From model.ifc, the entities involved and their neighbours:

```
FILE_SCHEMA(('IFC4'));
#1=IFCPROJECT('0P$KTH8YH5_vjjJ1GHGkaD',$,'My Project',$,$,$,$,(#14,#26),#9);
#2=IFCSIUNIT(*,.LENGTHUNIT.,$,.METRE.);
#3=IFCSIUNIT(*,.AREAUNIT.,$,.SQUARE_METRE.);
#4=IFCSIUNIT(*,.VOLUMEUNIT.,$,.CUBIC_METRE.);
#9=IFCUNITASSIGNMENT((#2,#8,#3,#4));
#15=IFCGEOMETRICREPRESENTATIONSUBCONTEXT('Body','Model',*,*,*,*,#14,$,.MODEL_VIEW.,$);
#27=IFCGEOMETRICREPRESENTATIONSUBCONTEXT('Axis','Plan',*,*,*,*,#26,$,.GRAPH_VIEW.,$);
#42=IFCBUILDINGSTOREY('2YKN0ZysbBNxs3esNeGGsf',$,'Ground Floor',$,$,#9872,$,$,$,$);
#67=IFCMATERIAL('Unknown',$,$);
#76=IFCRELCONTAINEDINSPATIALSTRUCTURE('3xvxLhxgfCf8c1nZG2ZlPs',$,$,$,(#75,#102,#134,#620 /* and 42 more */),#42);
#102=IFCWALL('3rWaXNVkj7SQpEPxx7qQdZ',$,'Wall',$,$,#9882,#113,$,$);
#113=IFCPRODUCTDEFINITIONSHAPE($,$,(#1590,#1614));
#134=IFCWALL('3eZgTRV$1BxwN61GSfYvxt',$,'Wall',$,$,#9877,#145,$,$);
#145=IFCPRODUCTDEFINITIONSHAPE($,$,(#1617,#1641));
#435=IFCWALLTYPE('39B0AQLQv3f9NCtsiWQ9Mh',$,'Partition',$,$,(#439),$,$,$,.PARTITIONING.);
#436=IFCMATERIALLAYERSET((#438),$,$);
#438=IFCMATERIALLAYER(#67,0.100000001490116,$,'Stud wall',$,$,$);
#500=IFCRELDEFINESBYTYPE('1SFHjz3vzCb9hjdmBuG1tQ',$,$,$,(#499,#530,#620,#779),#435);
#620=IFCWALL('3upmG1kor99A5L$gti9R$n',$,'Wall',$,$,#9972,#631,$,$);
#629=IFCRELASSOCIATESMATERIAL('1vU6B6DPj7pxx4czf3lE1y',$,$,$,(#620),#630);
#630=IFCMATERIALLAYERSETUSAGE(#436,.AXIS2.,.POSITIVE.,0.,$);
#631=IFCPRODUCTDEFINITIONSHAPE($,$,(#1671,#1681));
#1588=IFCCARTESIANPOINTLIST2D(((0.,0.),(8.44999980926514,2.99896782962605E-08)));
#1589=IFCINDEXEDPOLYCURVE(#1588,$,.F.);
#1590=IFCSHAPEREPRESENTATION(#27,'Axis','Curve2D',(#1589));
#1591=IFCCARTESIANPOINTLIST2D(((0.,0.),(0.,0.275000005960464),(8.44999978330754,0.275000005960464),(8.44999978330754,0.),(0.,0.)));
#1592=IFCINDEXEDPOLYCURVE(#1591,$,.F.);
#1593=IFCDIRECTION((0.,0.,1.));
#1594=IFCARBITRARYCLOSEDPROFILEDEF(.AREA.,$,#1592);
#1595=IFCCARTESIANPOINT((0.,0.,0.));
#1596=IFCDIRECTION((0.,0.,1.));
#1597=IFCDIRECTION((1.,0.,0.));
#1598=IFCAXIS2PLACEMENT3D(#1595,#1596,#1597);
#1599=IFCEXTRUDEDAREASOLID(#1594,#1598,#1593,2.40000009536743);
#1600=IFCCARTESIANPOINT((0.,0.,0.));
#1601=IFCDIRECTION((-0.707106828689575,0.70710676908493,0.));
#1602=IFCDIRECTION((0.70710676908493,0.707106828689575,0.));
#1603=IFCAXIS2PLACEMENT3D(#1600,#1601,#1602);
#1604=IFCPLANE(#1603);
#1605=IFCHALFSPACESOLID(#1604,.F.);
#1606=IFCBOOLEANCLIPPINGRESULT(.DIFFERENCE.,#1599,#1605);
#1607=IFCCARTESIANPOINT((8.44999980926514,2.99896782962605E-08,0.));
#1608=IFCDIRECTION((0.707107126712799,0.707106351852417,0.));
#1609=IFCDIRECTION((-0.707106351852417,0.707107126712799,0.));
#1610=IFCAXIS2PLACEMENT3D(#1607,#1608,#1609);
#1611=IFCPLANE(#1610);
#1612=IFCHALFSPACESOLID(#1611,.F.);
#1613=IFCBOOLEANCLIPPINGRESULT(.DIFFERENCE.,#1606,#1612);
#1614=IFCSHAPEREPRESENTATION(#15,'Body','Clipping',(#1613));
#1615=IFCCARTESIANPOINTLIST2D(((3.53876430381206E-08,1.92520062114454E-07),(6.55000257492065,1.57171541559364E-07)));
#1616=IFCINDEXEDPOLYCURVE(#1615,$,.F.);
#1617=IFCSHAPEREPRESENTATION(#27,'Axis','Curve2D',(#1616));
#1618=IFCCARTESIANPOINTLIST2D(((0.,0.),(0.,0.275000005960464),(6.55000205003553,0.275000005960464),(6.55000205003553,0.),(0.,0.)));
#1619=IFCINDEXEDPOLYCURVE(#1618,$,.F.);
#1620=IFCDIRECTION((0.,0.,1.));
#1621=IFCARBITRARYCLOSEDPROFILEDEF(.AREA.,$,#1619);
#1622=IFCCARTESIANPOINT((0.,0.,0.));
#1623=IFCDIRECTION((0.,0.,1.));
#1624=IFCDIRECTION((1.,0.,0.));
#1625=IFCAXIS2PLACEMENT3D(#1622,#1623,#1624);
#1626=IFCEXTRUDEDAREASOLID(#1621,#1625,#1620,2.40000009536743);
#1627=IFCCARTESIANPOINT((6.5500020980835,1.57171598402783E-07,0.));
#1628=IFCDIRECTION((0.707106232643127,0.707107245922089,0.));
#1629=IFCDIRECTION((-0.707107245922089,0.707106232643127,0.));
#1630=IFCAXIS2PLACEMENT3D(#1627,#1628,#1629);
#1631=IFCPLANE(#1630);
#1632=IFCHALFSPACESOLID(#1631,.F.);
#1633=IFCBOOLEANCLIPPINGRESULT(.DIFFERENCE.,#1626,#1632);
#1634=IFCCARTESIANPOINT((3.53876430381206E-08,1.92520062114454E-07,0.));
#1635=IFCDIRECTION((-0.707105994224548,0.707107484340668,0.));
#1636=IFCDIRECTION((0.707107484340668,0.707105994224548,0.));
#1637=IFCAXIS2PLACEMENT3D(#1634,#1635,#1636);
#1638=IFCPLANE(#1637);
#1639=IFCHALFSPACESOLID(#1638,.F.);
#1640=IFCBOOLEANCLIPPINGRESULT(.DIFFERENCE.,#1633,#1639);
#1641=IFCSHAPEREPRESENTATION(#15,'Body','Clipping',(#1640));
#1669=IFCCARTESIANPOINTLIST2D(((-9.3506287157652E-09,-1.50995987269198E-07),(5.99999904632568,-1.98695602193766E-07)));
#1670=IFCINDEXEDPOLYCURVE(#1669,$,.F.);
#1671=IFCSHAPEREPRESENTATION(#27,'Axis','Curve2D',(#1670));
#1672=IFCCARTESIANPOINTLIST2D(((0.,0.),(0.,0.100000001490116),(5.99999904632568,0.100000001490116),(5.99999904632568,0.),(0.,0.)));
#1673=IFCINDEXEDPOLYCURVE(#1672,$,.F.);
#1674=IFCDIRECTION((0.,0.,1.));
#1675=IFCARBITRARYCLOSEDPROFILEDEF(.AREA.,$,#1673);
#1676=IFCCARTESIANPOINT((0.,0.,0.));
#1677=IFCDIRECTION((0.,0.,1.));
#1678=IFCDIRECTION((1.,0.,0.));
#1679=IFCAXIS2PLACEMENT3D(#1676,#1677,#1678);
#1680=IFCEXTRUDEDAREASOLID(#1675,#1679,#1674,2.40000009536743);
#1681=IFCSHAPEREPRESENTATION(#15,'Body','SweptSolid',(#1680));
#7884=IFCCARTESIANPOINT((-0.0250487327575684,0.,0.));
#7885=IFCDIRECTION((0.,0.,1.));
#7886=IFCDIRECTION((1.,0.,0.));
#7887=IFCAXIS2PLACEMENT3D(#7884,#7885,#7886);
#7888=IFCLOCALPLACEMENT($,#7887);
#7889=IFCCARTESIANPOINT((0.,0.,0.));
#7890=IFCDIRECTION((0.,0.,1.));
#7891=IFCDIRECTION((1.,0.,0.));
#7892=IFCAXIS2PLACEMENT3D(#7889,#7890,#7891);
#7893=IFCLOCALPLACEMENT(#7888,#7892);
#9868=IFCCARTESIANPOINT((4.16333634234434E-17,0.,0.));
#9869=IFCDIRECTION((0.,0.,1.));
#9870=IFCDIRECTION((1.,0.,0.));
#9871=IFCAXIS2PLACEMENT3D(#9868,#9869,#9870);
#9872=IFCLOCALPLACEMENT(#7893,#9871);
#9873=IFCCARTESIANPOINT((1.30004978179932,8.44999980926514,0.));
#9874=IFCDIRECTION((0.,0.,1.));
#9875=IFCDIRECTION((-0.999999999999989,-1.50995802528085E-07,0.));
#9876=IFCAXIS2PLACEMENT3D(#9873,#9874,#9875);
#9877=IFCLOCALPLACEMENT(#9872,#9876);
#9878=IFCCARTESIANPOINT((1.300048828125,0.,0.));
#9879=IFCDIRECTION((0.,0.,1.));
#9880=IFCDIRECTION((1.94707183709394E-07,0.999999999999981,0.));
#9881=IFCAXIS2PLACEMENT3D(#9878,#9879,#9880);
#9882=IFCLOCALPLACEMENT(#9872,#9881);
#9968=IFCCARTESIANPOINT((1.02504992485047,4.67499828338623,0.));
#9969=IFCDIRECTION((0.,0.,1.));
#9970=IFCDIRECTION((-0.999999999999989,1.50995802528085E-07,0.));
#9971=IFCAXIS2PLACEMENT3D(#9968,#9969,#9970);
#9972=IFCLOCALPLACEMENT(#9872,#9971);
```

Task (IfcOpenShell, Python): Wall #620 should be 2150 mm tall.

```python
import ifcopenshell
import ifcopenshell.geom
import ifcopenshell.util.representation
import ifcopenshell.util.shape
import ifcopenshell.util.unit

model = ifcopenshell.open("model.ifc")
unit_scale = ifcopenshell.util.unit.calculate_unit_scale(model)
settings = ifcopenshell.geom.settings()


def volume(element):
    """Net volume in cubic metres, openings subtracted."""
    shape = ifcopenshell.geom.create_shape(settings, element)
    return ifcopenshell.util.shape.get_volume(shape.geometry)


wall = model.by_guid("3upmG1kor99A5L$gti9R$n")
before = volume(wall)

body = ifcopenshell.util.representation.get_representation(wall, "Model", "Body")
solid = body.Items[0]
old_height = solid.Depth
solid.Depth = 2.15 / unit_scale
after = volume(wall)

print(f"height {old_height:g} -> {solid.Depth:g}, volume {before:.3f} -> {after:.3f} m3")

model.write("model_v2.ifc")
```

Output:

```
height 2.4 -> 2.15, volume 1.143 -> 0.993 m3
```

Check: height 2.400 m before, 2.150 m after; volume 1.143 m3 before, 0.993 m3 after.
